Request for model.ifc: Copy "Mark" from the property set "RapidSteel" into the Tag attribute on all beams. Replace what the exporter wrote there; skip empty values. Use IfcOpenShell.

First a look at what the model holds.

```python
import ifcopenshell
import ifcopenshell.util.element

model = ifcopenshell.open("model.ifc")
print(model.schema)
beams = model.by_type("IfcBeam")
print(len(beams), "beams")
for e in beams[:8]:
    source = ifcopenshell.util.element.get_pset(e, "RapidSteel", "Mark")
    target = e.Tag
    print(e.id(), repr(source), repr(target), sep=" | ")
```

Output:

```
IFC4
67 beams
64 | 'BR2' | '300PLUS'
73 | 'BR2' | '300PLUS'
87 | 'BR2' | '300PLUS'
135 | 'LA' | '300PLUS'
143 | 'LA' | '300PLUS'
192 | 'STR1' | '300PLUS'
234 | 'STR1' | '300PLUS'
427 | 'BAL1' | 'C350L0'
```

```python
import ifcopenshell
import ifcopenshell.util.element

model = ifcopenshell.open("model.ifc")

count = 0
for e in model.by_type("IfcBeam"):
    value = ifcopenshell.util.element.get_pset(e, "RapidSteel", "Mark")
    current = e.Tag
    if not value or not value.strip() or current == value:
        continue
    e.Tag = value
    count += 1

print(count, "beams updated")

model.write("model_updated.ifc")
```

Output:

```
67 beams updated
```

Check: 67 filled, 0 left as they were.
